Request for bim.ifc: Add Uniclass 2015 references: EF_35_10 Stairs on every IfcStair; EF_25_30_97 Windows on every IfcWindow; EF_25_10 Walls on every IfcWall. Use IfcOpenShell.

First a look at what the model holds.

```python
import ifcopenshell

model = ifcopenshell.open("bim.ifc")
print(model.schema)
print("classifications:", [c.Name for c in model.by_type("IfcClassification")])
for ifc_class in ("IfcDoor", "IfcRoof", "IfcStair", "IfcWall", "IfcWindow"):
    print(ifc_class, len(model.by_type(ifc_class)))
```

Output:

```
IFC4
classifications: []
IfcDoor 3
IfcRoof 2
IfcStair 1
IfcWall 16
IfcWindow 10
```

```python
import ifcopenshell
import ifcopenshell.api.classification

model = ifcopenshell.open("bim.ifc")

system = ifcopenshell.api.classification.add_classification(model, classification="Uniclass 2015")

codes = {
    "IfcStair": ("EF_35_10", "Stairs"),
    "IfcWindow": ("EF_25_30_97", "Windows"),
    "IfcWall": ("EF_25_10", "Walls"),
}
for ifc_class, (code, name) in codes.items():
    products = model.by_type(ifc_class)
    ifcopenshell.api.classification.add_reference(
        model, products=products, classification=system, identification=code, name=name
    )
    print(code, len(products))

model.write("bim_updated.ifc")
```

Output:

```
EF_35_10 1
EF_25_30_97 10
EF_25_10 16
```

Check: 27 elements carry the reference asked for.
